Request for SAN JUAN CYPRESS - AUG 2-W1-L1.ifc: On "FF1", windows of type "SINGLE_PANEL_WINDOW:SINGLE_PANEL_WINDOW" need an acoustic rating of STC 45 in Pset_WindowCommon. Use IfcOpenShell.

First a look at what the model holds.

```python
import ifcopenshell
import ifcopenshell.util.element

model = ifcopenshell.open("SAN JUAN CYPRESS - AUG 2-W1-L1.ifc")
print(model.schema)
storey = next(s for s in model.by_type("IfcBuildingStorey") if s.Name == "FF1")
windows = [e for e in ifcopenshell.util.element.get_decomposition(storey) if e.is_a("IfcWindow")]
seen = {}
for e in windows:
    element_type = ifcopenshell.util.element.get_type(e)
    key = (element_type.Name if element_type != e and element_type else None, ifcopenshell.util.element.get_pset(e, "Pset_WindowCommon", "AcousticRating"))
    seen[key] = seen.get(key, 0) + 1
for (name, value), count in sorted(seen.items(), key=str):
    print(count, "x", name, "|", value)
```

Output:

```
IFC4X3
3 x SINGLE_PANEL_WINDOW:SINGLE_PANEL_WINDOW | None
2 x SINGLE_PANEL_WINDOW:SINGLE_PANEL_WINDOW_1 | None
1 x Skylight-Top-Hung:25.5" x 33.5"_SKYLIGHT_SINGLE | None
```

```python
import ifcopenshell
import ifcopenshell.api.pset
import ifcopenshell.util.element

model = ifcopenshell.open("SAN JUAN CYPRESS - AUG 2-W1-L1.ifc")

storey = next(s for s in model.by_type("IfcBuildingStorey") if s.Name == "FF1")
windows = [e for e in ifcopenshell.util.element.get_decomposition(storey) if e.is_a("IfcWindow")]

count = 0
for e in windows:
    element_type = ifcopenshell.util.element.get_type(e)
    if element_type in (None, e) or element_type.Name != "SINGLE_PANEL_WINDOW:SINGLE_PANEL_WINDOW":
        continue
    # add_pset returns the element's existing set when there is one.
    pset = ifcopenshell.api.pset.add_pset(model, product=e, name="Pset_WindowCommon")
    ifcopenshell.api.pset.edit_pset(model, pset=pset, properties={"AcousticRating": "STC 45"})
    count += 1

print(count, "windows updated")

model.write("SAN JUAN CYPRESS - AUG 2-W1-L1_updated.ifc")
```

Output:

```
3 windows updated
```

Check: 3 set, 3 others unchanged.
